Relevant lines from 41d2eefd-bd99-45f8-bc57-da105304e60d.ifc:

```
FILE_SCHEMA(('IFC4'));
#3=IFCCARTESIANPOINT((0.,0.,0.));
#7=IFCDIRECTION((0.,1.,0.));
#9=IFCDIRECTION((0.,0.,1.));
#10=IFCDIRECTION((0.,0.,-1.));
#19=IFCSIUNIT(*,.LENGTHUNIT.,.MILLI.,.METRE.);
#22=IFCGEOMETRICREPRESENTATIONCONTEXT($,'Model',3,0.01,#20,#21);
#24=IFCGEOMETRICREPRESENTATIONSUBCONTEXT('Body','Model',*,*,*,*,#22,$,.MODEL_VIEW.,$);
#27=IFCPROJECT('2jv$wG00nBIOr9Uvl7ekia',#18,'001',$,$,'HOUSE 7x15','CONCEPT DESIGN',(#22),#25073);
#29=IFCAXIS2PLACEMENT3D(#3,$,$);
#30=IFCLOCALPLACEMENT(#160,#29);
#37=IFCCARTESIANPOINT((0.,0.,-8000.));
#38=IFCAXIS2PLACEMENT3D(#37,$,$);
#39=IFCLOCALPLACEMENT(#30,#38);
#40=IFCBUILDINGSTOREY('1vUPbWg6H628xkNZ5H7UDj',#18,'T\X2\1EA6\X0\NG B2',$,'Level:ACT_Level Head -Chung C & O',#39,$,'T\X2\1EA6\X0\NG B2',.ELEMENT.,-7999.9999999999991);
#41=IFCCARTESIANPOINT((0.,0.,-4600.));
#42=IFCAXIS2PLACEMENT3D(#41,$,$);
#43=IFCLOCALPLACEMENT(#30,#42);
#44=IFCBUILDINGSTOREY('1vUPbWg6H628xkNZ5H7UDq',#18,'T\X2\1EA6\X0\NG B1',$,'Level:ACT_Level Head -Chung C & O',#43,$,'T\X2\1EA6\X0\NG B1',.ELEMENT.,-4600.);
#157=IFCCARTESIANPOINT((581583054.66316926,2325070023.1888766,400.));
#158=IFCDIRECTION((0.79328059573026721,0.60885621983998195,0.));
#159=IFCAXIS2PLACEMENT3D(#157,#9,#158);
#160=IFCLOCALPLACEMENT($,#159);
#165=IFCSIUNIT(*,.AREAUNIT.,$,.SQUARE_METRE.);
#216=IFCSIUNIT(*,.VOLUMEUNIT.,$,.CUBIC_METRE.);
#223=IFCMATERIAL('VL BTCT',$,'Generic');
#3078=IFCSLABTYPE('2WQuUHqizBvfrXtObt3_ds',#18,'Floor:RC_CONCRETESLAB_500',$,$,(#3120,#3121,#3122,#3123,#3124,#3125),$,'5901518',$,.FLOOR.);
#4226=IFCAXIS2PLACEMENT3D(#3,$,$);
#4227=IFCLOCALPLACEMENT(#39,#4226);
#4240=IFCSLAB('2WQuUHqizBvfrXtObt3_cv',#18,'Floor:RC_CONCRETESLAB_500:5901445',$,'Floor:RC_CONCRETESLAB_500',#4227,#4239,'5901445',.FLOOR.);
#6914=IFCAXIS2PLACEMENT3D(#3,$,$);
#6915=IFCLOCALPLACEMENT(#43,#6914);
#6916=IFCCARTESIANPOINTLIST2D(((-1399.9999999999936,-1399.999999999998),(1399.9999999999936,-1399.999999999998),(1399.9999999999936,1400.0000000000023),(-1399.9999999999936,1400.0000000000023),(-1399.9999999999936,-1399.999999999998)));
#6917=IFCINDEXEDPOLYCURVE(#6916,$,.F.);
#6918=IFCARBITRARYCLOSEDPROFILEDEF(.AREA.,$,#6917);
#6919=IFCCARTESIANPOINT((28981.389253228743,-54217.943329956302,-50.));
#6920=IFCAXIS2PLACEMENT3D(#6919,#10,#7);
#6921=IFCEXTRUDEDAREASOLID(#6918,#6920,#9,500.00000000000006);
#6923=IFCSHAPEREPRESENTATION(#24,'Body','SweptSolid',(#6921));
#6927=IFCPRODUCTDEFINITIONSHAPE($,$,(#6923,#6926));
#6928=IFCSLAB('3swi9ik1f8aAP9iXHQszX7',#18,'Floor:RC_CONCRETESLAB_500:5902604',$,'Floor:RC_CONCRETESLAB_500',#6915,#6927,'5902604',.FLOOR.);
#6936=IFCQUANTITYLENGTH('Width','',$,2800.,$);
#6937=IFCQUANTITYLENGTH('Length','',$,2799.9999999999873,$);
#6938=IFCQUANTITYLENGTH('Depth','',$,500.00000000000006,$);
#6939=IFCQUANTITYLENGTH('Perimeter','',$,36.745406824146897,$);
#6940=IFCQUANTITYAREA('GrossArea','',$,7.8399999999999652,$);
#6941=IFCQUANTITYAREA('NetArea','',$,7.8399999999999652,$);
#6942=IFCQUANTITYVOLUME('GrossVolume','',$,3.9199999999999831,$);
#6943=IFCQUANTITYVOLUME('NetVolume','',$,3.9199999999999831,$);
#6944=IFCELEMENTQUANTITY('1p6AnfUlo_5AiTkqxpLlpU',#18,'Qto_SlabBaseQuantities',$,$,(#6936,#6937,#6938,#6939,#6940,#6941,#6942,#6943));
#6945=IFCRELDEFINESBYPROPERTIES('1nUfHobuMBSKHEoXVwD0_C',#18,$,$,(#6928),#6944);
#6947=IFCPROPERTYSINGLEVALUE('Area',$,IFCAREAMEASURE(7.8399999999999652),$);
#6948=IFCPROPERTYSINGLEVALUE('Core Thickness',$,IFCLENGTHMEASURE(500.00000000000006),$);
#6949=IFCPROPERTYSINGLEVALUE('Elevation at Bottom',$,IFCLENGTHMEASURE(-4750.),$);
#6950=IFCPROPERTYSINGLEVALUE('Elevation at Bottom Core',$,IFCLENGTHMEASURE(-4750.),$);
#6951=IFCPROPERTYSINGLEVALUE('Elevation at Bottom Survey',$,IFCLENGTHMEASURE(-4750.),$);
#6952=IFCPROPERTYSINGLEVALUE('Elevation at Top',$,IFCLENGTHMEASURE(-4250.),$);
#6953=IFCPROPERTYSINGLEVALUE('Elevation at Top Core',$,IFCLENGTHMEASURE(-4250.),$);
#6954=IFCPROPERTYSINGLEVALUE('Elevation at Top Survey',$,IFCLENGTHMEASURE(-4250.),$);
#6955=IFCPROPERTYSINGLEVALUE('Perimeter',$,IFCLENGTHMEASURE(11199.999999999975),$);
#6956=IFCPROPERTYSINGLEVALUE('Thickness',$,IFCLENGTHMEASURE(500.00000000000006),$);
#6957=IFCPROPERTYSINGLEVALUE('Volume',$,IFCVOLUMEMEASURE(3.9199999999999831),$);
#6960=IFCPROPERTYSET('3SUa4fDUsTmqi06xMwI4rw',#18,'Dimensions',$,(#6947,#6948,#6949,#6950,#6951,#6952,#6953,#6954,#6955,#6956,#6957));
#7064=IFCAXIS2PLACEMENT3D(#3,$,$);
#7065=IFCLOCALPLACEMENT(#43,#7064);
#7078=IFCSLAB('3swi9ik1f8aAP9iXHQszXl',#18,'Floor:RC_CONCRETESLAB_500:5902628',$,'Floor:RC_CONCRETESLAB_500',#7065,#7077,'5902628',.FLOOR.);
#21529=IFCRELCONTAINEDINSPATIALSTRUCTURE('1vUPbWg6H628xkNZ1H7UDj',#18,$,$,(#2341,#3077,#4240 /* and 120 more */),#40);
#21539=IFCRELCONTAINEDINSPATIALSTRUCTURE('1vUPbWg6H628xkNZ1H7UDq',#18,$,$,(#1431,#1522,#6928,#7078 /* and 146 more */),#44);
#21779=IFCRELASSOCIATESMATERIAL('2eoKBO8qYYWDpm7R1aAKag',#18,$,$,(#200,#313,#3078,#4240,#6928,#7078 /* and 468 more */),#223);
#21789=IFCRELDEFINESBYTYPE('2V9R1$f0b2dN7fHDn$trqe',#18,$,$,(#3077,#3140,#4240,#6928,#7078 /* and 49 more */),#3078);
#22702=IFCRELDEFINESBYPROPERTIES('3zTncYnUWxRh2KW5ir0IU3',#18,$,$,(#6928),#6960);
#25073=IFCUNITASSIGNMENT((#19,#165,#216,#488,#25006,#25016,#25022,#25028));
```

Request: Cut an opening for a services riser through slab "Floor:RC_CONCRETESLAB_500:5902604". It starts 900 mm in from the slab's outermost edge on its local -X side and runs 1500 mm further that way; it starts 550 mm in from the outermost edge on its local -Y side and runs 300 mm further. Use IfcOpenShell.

```python
import numpy as np
import ifcopenshell
import ifcopenshell.api.feature
import ifcopenshell.api.geometry
import ifcopenshell.api.pset
import ifcopenshell.api.root
import ifcopenshell.geom
import ifcopenshell.util.element
import ifcopenshell.util.placement
import ifcopenshell.util.representation
import ifcopenshell.util.shape
import ifcopenshell.util.unit

model = ifcopenshell.open("41d2eefd-bd99-45f8-bc57-da105304e60d.ifc")
unit_scale = ifcopenshell.util.unit.calculate_unit_scale(model)
area_scale = ifcopenshell.util.unit.calculate_unit_scale(model, "AREAUNIT")
volume_scale = ifcopenshell.util.unit.calculate_unit_scale(model, "VOLUMEUNIT")
settings = ifcopenshell.geom.settings()


def volume(element):
    """Net volume in cubic metres, openings subtracted."""
    shape = ifcopenshell.geom.create_shape(settings, element)
    return ifcopenshell.util.shape.get_volume(shape.geometry)


slab = model.by_guid("3swi9ik1f8aAP9iXHQszX7")
before = volume(slab)

# Extent in the slab's own axes, in metres. The edges named are its -X and -Y sides.
slab_shape = ifcopenshell.geom.create_shape(settings, slab)
vertices = ifcopenshell.util.shape.get_vertices(slab_shape.geometry)
x_min, y_min, bottom = vertices.min(axis=0)
top = vertices[:, 2].max()

opening = ifcopenshell.api.root.create_entity(model, ifc_class="IfcOpeningElement", name="Services riser opening", predefined_type="OPENING")
context = ifcopenshell.util.representation.get_context(model, "Model", "Body", "MODEL_VIEW")
width, depth = 1.5, 0.3
outline = [(0.0, 0.0), (width, 0.0), (width, depth), (0.0, depth), (0.0, 0.0)]
# Overshoot both faces by 50 mm so the cut is clean.
shape = ifcopenshell.api.geometry.add_slab_representation(
    model, context=context, depth=top - bottom + 0.1, polyline=outline
)
ifcopenshell.api.geometry.assign_representation(model, product=opening, representation=shape)

matrix = ifcopenshell.util.placement.get_local_placement(slab.ObjectPlacement)
matrix[:, 3] = matrix @ np.append(np.array([x_min + 0.9, y_min + 0.55, bottom - 0.05]) / unit_scale, 1.0)
ifcopenshell.api.geometry.edit_object_placement(model, product=opening, matrix=matrix, is_si=False)
ifcopenshell.api.feature.add_feature(model, feature=opening, element=slab)

after = volume(slab)

# Update the slab's stored quantities.
qto = model.by_id(ifcopenshell.util.element.get_pset(slab, "Qto_SlabBaseQuantities", should_inherit=False)["id"])
ifcopenshell.api.pset.edit_qto(model, qto=qto, properties={
    "NetArea": after / (top - bottom) / area_scale,
    "NetVolume": after / volume_scale,
})
pset = model.by_id(ifcopenshell.util.element.get_pset(slab, "Dimensions", should_inherit=False)["id"])
ifcopenshell.api.pset.edit_pset(model, pset=pset, properties={
    "Area": model.create_entity("IfcAreaMeasure", after / (top - bottom) / area_scale),
    "Volume": model.create_entity("IfcVolumeMeasure", after / volume_scale),
})

print(f"slab volume {before:.3f} -> {after:.3f} m3")

model.write("41d2eefd-bd99-45f8-bc57-da105304e60d_rev.ifc")
```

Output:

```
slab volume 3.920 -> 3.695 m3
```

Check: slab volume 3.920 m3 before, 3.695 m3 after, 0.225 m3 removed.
